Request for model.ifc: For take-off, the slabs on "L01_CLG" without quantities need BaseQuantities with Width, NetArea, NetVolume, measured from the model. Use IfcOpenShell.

First a look at what the model holds.

```python
import ifcopenshell
import ifcopenshell.util.element
import ifcopenshell.util.unit

model = ifcopenshell.open("model.ifc")
print(model.schema)
for unit_type in ("LENGTHUNIT", "AREAUNIT", "VOLUMEUNIT"):
    print(unit_type, ifcopenshell.util.unit.calculate_unit_scale(model, unit_type))
storey = next(s for s in model.by_type("IfcBuildingStorey") if s.Name == "L01_CLG")
slabs = [e for e in ifcopenshell.util.element.get_decomposition(storey) if e.is_a("IfcSlab")]
for e in sorted(slabs, key=lambda e: e.id()):
    print(e.id(), e.is_a(), e.Name, list(ifcopenshell.util.element.get_psets(e, qtos_only=True)), sep=" | ")
```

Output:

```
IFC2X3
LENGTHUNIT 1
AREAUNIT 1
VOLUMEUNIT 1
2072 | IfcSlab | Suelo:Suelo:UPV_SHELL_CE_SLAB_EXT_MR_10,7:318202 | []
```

```python
import ifcopenshell
import ifcopenshell.api.pset
import ifcopenshell.geom
import ifcopenshell.util.element
import ifcopenshell.util.shape
import ifcopenshell.util.unit

model = ifcopenshell.open("model.ifc")
unit_scale = ifcopenshell.util.unit.calculate_unit_scale(model)
area_scale = ifcopenshell.util.unit.calculate_unit_scale(model, "AREAUNIT")
volume_scale = ifcopenshell.util.unit.calculate_unit_scale(model, "VOLUMEUNIT")
settings = ifcopenshell.geom.settings()

storey = next(s for s in model.by_type("IfcBuildingStorey") if s.Name == "L01_CLG")
slabs = [e for e in ifcopenshell.util.element.get_decomposition(storey) if e.is_a("IfcSlab")]

for e in sorted(slabs, key=lambda e: e.id()):
    if ifcopenshell.util.element.get_psets(e, qtos_only=True, should_inherit=False):
        continue
    # Geometry comes back in metres, in the element's own axes.
    shape = ifcopenshell.geom.create_shape(settings, e)
    values = {
        "Width": ifcopenshell.util.shape.get_z(shape.geometry) / unit_scale,
        "NetArea": ifcopenshell.util.shape.get_footprint_area(shape.geometry) / area_scale,
        "NetVolume": ifcopenshell.util.shape.get_volume(shape.geometry) / volume_scale,
    }
    qto = ifcopenshell.api.pset.add_qto(model, product=e, name="BaseQuantities")
    ifcopenshell.api.pset.edit_qto(model, qto=qto, properties=values)
    print(e.id(), {k: round(v, 3) for k, v in values.items()})

model.write("model_v2.ifc")
```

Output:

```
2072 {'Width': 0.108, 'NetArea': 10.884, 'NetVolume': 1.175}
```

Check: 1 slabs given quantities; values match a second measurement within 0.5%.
